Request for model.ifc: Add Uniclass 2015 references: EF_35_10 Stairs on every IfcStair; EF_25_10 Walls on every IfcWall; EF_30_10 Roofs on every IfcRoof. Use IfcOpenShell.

First a look at what the model holds.

```python
import ifcopenshell

model = ifcopenshell.open("model.ifc")
print(model.schema)
print("classifications:", [c.Name for c in model.by_type("IfcClassification")])
for ifc_class in ("IfcDoor", "IfcRoof", "IfcStair", "IfcWall", "IfcWindow"):
    print(ifc_class, len(model.by_type(ifc_class)))
```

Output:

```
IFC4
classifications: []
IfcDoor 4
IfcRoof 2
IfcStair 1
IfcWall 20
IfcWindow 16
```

```python
import ifcopenshell
import ifcopenshell.api.classification

model = ifcopenshell.open("model.ifc")

system = ifcopenshell.api.classification.add_classification(model, classification="Uniclass 2015")

codes = {
    "IfcStair": ("EF_35_10", "Stairs"),
    "IfcWall": ("EF_25_10", "Walls"),
    "IfcRoof": ("EF_30_10", "Roofs"),
}
for ifc_class, (code, name) in codes.items():
    products = model.by_type(ifc_class)
    ifcopenshell.api.classification.add_reference(
        model, products=products, classification=system, identification=code, name=name
    )
    print(code, len(products))

model.write("model_v2.ifc")
```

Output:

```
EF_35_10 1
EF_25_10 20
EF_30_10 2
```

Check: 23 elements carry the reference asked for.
